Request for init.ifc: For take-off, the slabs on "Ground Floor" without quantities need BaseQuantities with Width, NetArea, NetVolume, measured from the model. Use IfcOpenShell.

First a look at what the model holds.

```python
import ifcopenshell
import ifcopenshell.util.element
import ifcopenshell.util.unit

model = ifcopenshell.open("init.ifc")
print(model.schema)
for unit_type in ("LENGTHUNIT", "AREAUNIT", "VOLUMEUNIT"):
    print(unit_type, ifcopenshell.util.unit.calculate_unit_scale(model, unit_type))
storey = next(s for s in model.by_type("IfcBuildingStorey") if s.Name == "Ground Floor")
slabs = [e for e in ifcopenshell.util.element.get_decomposition(storey) if e.is_a("IfcSlab")]
for e in sorted(slabs, key=lambda e: e.id()):
    print(e.id(), e.is_a(), e.Name, list(ifcopenshell.util.element.get_psets(e, qtos_only=True)), sep=" | ")
```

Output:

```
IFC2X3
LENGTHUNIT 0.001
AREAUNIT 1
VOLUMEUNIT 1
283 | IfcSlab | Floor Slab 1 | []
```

```python
import ifcopenshell
import ifcopenshell.api.pset
import ifcopenshell.geom
import ifcopenshell.util.element
import ifcopenshell.util.shape
import ifcopenshell.util.unit

model = ifcopenshell.open("init.ifc")
unit_scale = ifcopenshell.util.unit.calculate_unit_scale(model)
area_scale = ifcopenshell.util.unit.calculate_unit_scale(model, "AREAUNIT")
volume_scale = ifcopenshell.util.unit.calculate_unit_scale(model, "VOLUMEUNIT")
settings = ifcopenshell.geom.settings()

storey = next(s for s in model.by_type("IfcBuildingStorey") if s.Name == "Ground Floor")
slabs = [e for e in ifcopenshell.util.element.get_decomposition(storey) if e.is_a("IfcSlab")]

for e in sorted(slabs, key=lambda e: e.id()):
    if ifcopenshell.util.element.get_psets(e, qtos_only=True, should_inherit=False):
        continue
    # Geometry comes back in metres, in the element's own axes.
    shape = ifcopenshell.geom.create_shape(settings, e)
    values = {
        "Width": ifcopenshell.util.shape.get_z(shape.geometry) / unit_scale,
        "NetArea": ifcopenshell.util.shape.get_footprint_area(shape.geometry) / area_scale,
        "NetVolume": ifcopenshell.util.shape.get_volume(shape.geometry) / volume_scale,
    }
    qto = ifcopenshell.api.pset.add_qto(model, product=e, name="BaseQuantities")
    ifcopenshell.api.pset.edit_qto(model, qto=qto, properties=values)
    print(e.id(), {k: round(v, 3) for k, v in values.items()})

model.write("init_edited.ifc")
```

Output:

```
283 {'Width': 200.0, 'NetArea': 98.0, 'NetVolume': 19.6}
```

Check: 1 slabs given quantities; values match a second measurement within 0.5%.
